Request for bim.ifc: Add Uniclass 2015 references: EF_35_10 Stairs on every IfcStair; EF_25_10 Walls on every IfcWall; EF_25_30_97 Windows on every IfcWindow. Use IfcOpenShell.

First a look at what the model holds.

```python
import ifcopenshell

model = ifcopenshell.open("bim.ifc")
print(model.schema)
print("classifications:", [c.Name for c in model.by_type("IfcClassification")])
for ifc_class in ("IfcDoor", "IfcRoof", "IfcStair", "IfcWall", "IfcWindow"):
    print(ifc_class, len(model.by_type(ifc_class)))
```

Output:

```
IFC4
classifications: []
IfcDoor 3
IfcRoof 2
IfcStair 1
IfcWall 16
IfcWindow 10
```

```python
import ifcopenshell
import ifcopenshell.api.classification

model = ifcopenshell.open("bim.ifc")

system = ifcopenshell.api.classification.add_classification(model, classification="Uniclass 2015")

codes = {
    "IfcStair": ("EF_35_10", "Stairs"),
    "IfcWall": ("EF_25_10", "Walls"),
    "IfcWindow": ("EF_25_30_97", "Windows"),
}
for ifc_class, (code, name) in codes.items():
    products = model.by_type(ifc_class)
    ifcopenshell.api.classification.add_reference(
        model, products=products, classification=system, identification=code, name=name
    )
    print(code, len(products))

model.write("bim-out.ifc")
```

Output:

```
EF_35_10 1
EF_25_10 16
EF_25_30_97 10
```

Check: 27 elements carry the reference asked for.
